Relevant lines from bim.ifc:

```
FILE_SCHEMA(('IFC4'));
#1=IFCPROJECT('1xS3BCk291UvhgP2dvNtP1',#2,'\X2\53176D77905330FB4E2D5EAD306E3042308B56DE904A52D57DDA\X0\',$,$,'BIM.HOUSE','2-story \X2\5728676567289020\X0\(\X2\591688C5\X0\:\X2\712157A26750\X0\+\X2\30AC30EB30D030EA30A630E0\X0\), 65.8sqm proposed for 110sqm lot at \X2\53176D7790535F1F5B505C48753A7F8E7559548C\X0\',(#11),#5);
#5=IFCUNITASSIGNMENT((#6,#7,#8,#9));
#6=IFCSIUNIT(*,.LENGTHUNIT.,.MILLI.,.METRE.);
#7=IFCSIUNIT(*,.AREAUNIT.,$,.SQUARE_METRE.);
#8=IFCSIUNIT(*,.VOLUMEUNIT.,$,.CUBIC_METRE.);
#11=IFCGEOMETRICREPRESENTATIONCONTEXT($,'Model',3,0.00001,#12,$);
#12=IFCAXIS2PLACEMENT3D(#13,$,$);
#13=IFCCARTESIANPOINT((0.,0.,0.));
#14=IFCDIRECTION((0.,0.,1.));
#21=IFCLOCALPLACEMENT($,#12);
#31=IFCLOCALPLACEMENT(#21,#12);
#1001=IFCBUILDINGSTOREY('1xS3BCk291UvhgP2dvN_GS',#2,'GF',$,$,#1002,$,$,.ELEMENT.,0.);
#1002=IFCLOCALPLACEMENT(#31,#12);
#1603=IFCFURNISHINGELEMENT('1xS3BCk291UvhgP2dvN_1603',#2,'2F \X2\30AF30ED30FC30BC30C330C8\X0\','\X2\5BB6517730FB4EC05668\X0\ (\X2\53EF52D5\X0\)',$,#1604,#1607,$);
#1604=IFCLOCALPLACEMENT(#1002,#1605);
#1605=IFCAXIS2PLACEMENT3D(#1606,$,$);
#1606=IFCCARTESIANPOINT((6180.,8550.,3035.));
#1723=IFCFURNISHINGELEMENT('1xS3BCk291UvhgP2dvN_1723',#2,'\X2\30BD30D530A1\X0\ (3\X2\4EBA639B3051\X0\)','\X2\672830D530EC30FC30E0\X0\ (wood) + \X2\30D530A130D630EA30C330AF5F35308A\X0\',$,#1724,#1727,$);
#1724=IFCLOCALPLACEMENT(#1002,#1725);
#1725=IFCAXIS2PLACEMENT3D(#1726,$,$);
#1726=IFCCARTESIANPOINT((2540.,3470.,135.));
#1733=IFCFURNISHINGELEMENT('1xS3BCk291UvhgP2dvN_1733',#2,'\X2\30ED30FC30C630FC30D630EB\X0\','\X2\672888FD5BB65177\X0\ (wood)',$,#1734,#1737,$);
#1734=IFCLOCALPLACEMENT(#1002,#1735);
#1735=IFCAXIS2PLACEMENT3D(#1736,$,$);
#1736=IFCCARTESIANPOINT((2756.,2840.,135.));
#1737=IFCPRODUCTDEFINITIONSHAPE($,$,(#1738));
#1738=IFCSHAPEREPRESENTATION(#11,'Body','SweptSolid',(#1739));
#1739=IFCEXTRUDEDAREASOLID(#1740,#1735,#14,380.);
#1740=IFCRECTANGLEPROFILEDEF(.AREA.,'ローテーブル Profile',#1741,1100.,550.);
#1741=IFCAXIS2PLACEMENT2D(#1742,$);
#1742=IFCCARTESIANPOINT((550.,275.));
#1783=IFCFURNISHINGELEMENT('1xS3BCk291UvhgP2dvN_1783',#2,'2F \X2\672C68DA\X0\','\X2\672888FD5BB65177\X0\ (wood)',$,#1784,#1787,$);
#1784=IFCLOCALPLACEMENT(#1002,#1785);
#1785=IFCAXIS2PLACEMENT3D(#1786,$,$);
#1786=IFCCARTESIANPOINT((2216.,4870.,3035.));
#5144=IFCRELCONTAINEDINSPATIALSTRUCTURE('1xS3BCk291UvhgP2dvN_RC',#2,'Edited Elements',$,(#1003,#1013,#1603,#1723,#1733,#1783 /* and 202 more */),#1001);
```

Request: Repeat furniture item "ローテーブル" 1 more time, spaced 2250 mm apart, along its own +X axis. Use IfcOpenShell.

```python
import ifcopenshell
import ifcopenshell.api.geometry
import ifcopenshell.api.root
import ifcopenshell.util.element
import ifcopenshell.util.placement
import ifcopenshell.util.unit

model = ifcopenshell.open("bim.ifc")
unit_scale = ifcopenshell.util.unit.calculate_unit_scale(model)


def reuse_history(source, copy):
    """copy_class also copies each property set's owner history, people and application; keep the originals."""
    for rel in copy.IsDefinedBy:
        if rel.is_a("IfcRelDefinesByProperties") and (history := rel.RelatingPropertyDefinition.OwnerHistory):
            rel.RelatingPropertyDefinition.OwnerHistory = source.OwnerHistory
            ifcopenshell.util.element.remove_deep2(model, history)


source = model.by_guid("1xS3BCk291UvhgP2dvN_1733")
base = ifcopenshell.util.placement.get_local_placement(source.ObjectPlacement)
step = base[:3, 0] * 2.25 / unit_scale

for i in range(1, 2):
    copy = ifcopenshell.api.root.copy_class(model, product=source)
    copy.Representation = ifcopenshell.util.element.copy_deep(
        model, source.Representation, exclude=["IfcGeometricRepresentationContext", "IfcRepresentationMap"]
    )
    reuse_history(source, copy)
    matrix = base.copy()
    matrix[:3, 3] += i * step
    print("added at", matrix[:3, 3].round(3) + 0.0)
    ifcopenshell.api.geometry.edit_object_placement(model, product=copy, matrix=matrix, is_si=False)

model.write("bim_rev.ifc")
```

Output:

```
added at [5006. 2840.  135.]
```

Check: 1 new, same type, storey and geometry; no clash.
